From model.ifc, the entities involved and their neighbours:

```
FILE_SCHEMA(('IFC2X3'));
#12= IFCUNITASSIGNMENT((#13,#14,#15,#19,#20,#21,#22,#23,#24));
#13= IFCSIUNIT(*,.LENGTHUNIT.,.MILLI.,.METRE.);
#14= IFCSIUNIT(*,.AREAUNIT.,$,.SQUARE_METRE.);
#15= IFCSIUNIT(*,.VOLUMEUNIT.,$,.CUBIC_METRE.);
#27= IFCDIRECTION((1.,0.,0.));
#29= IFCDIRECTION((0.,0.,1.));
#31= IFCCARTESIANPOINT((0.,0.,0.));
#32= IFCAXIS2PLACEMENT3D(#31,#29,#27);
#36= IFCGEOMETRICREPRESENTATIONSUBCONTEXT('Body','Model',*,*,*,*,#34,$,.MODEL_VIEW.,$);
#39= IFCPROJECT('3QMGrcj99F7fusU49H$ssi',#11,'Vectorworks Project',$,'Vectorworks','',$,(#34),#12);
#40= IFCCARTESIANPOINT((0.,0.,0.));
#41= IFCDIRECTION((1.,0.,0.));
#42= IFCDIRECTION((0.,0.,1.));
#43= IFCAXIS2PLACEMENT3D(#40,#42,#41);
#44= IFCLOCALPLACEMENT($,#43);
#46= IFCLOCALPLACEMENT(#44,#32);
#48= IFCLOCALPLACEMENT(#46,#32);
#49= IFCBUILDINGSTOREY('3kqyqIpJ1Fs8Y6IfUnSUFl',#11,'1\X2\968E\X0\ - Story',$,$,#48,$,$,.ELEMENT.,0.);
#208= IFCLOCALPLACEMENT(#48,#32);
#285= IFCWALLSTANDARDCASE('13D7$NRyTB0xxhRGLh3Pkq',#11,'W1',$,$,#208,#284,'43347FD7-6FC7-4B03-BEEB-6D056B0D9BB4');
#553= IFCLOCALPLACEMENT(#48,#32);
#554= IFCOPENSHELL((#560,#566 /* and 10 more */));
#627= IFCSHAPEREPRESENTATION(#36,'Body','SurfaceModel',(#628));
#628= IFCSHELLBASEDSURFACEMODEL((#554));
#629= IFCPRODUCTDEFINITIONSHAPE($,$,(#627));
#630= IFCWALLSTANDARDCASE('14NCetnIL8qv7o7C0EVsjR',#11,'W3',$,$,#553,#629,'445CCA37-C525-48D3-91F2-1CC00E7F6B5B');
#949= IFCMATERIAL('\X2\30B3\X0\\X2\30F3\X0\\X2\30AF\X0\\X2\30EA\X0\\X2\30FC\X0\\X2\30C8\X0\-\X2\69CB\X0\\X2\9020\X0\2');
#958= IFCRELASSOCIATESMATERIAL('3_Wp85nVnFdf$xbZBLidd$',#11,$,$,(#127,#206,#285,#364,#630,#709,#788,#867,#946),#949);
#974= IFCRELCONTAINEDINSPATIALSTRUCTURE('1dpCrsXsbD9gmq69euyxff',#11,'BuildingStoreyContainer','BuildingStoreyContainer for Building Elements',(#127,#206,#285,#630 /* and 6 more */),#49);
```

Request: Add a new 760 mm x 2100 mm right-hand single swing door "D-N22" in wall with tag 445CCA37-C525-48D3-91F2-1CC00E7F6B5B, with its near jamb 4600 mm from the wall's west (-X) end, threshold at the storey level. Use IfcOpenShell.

```python
import numpy as np
import ifcopenshell
import ifcopenshell.api.feature
import ifcopenshell.api.geometry
import ifcopenshell.api.root
import ifcopenshell.api.spatial
import ifcopenshell.api.type
import ifcopenshell.geom
import ifcopenshell.util.element
import ifcopenshell.util.placement
import ifcopenshell.util.representation
import ifcopenshell.util.shape
import ifcopenshell.util.unit

model = ifcopenshell.open("model.ifc")
unit_scale = ifcopenshell.util.unit.calculate_unit_scale(model)
settings = ifcopenshell.geom.settings()


def volume(element):
    """Net volume in cubic metres, openings subtracted."""
    shape = ifcopenshell.geom.create_shape(settings, element)
    return ifcopenshell.util.shape.get_volume(shape.geometry)


wall = model.by_guid("14NCetnIL8qv7o7C0EVsjR")
storey = ifcopenshell.util.element.get_container(wall, ifc_class="IfcBuildingStorey")
context = ifcopenshell.util.representation.get_context(model, "Model", "Body", "MODEL_VIEW")
before = volume(wall)

width, height, from_end, sill = 0.76, 2.1, 4.6, 0.0  # metres

# The wall runs along its own X axis, and the end named is its -X end.
wall_shape = ifcopenshell.geom.create_shape(settings, wall)
x, y, z = ifcopenshell.util.shape.get_vertices(wall_shape.geometry).T
start = x.min() + from_end
face, thickness = float(y.min()), float(y.max() - y.min())
wall_matrix = ifcopenshell.util.placement.get_local_placement(wall.ObjectPlacement)
level = ifcopenshell.util.placement.get_local_placement(storey.ObjectPlacement)[2, 3]


def in_wall(x, y):
    """Placement at x, y metres in the wall's axes, at sill height."""
    matrix = wall_matrix.copy()
    matrix[:, 3] = wall_matrix @ np.array([x / unit_scale, y / unit_scale, 0.0, 1.0])
    matrix[2, 3] = level + sill / unit_scale
    return matrix


# Opening: a box that overshoots both wall faces by 50 mm.
opening = ifcopenshell.api.root.create_entity(model, ifc_class="IfcOpeningElement")
box = ifcopenshell.api.geometry.add_wall_representation(
    model, context=context, length=width, height=height, thickness=thickness + 0.1
)
ifcopenshell.api.geometry.assign_representation(model, product=opening, representation=box)
ifcopenshell.api.geometry.edit_object_placement(model, product=opening, matrix=in_wall(start, face - 0.05), is_si=False)
ifcopenshell.api.feature.add_feature(model, feature=opening, element=wall)

door = ifcopenshell.api.root.create_entity(model, ifc_class="IfcDoor", name="D-N22")
door.OverallWidth, door.OverallHeight = width / unit_scale, height / unit_scale
body = ifcopenshell.api.geometry.add_door_representation(
    model,
    context=context,
    overall_width=door.OverallWidth,
    overall_height=door.OverallHeight,
    operation_type="SINGLE_SWING_RIGHT",
    lining_properties={"LiningDepth": thickness / unit_scale, "ThresholdDepth": thickness / unit_scale},
)
ifcopenshell.api.geometry.assign_representation(model, product=door, representation=body)
ifcopenshell.api.spatial.assign_container(model, products=[door], relating_structure=storey)
fills = ifcopenshell.api.feature.add_filling(model, opening=opening, element=door)
fills.OwnerHistory = door.OwnerHistory  # required in IFC2X3

# IFC2X3 keeps the operation on the door style.
style = ifcopenshell.api.root.create_entity(model, ifc_class="IfcDoorStyle", name="D-N22")
style.OperationType, style.ConstructionType = "SINGLE_SWING_RIGHT", "NOTDEFINED"
style.ParameterTakesPrecedence = style.Sizeable = False
ifcopenshell.api.type.assign_type(model, related_objects=[door], relating_type=style)

# The lining spans the wall, so the door starts at the wall face.
ifcopenshell.api.geometry.edit_object_placement(model, product=door, matrix=in_wall(start, face), is_si=False)

after = volume(wall)

print(f"wall volume {before:.3f} -> {after:.3f} m3")

model.write("model_updated.ifc")
```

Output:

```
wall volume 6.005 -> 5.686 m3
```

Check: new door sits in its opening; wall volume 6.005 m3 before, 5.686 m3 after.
